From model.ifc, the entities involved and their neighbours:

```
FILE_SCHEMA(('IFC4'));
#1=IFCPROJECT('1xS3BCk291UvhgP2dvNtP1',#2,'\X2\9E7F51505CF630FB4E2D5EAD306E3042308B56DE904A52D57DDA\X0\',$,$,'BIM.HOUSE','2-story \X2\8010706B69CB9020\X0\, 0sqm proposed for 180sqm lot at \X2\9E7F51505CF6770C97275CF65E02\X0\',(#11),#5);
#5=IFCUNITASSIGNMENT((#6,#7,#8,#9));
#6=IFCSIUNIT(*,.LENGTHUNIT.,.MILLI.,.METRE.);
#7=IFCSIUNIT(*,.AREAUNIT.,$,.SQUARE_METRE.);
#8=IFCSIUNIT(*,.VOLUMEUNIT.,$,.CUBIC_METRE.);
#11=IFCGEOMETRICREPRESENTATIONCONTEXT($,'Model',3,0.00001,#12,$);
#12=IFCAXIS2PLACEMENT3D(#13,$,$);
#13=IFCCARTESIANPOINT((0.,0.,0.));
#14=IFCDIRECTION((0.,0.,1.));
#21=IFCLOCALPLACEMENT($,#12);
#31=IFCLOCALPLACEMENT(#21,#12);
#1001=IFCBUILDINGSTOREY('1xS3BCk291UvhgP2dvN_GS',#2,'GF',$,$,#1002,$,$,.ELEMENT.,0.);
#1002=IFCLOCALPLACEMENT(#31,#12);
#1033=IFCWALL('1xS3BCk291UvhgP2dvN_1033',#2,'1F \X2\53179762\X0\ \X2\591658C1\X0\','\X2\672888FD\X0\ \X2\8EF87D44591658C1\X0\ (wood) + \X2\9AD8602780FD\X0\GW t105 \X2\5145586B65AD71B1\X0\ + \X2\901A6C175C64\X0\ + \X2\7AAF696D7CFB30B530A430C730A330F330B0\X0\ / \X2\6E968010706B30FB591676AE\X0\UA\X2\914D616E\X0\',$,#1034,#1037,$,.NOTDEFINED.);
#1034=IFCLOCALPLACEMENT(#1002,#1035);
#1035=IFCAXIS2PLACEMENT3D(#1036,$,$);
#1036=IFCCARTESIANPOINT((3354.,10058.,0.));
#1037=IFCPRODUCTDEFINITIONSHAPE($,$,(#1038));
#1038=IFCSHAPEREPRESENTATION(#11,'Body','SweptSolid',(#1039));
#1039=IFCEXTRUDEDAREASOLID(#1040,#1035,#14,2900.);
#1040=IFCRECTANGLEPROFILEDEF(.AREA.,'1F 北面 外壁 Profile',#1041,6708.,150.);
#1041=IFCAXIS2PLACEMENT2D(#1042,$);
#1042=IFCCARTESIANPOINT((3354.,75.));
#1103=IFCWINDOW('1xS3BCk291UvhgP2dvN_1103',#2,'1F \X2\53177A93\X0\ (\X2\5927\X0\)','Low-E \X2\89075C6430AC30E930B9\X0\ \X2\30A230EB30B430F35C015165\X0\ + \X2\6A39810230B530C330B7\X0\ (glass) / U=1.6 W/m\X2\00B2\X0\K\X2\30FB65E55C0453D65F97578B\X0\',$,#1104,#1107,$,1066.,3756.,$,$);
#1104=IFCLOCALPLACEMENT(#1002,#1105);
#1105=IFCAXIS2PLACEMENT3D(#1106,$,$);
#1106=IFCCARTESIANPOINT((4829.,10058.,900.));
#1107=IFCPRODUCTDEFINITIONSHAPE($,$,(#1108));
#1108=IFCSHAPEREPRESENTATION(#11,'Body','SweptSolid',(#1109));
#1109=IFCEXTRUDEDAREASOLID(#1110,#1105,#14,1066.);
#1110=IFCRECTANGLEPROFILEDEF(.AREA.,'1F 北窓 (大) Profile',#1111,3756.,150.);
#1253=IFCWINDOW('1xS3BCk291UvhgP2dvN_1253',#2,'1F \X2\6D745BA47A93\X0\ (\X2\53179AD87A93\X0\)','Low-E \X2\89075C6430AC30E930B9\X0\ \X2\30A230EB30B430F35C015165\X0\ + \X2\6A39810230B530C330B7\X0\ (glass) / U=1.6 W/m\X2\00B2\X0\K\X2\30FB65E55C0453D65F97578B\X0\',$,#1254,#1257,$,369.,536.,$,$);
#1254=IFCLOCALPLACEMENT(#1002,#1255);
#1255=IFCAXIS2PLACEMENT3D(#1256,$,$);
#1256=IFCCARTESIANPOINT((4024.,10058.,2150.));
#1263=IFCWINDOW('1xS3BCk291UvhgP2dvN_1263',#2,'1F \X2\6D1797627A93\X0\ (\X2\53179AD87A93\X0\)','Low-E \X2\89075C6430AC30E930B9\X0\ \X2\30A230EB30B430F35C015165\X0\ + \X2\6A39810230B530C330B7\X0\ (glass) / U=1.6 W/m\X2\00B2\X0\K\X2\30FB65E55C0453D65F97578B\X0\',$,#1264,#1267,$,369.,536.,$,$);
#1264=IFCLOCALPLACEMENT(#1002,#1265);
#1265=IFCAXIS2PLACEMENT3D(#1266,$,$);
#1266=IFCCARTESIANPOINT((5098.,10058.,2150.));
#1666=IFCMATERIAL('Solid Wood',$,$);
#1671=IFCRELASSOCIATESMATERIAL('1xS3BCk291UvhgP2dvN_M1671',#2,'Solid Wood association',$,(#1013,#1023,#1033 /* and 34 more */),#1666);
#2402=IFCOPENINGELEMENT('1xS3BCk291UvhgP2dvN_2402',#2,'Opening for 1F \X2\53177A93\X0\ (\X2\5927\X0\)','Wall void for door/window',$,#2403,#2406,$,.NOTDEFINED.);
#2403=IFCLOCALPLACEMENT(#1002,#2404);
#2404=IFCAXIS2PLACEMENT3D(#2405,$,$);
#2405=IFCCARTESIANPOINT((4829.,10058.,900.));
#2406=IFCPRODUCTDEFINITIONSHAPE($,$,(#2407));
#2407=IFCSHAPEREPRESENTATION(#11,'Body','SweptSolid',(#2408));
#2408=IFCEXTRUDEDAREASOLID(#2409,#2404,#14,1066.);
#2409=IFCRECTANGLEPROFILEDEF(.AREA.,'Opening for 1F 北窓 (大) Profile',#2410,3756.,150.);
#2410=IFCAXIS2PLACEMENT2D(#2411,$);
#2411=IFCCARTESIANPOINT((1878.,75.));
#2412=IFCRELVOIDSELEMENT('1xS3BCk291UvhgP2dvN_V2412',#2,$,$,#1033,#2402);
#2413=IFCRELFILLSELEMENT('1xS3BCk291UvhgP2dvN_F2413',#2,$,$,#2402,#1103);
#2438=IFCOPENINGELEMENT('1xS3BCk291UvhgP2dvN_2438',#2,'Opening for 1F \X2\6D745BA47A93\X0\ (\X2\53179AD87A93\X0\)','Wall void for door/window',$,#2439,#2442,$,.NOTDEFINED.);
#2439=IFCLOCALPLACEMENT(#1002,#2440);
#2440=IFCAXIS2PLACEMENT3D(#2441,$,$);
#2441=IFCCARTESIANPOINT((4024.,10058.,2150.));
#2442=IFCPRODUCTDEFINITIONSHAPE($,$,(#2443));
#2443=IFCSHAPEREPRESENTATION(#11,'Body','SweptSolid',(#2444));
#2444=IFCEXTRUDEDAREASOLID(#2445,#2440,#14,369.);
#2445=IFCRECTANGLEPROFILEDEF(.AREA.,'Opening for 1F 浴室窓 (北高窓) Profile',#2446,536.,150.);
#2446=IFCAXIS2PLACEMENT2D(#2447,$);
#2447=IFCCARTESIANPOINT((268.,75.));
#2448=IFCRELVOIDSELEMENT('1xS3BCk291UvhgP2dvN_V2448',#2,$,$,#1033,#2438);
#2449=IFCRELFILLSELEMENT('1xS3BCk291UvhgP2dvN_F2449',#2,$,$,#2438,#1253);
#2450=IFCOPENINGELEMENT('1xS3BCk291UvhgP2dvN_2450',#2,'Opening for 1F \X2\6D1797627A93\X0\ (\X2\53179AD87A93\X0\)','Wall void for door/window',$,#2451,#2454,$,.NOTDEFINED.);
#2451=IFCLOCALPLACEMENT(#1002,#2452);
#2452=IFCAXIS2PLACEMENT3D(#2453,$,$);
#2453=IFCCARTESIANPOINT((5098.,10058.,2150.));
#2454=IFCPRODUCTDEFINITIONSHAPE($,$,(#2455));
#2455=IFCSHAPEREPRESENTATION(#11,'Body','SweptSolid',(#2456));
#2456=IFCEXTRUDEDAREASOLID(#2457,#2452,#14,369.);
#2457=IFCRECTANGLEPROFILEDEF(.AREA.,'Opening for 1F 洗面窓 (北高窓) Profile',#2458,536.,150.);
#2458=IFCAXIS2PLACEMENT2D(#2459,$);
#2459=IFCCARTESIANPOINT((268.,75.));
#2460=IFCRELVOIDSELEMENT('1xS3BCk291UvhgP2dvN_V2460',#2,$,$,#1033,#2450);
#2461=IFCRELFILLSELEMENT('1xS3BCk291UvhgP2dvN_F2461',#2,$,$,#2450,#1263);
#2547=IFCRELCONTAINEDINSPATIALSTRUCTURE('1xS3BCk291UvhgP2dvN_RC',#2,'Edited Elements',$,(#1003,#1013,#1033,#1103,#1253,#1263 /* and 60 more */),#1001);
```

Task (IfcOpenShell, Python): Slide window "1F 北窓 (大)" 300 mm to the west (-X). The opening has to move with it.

```python
import ifcopenshell
import ifcopenshell.api.geometry
import ifcopenshell.util.placement

model = ifcopenshell.open("model.ifc")

window = model.by_guid("1xS3BCk291UvhgP2dvN_1103")
opening = window.FillsVoids[0].RelatingOpeningElement
wall = opening.VoidsElements[0].RelatingBuildingElement

wall_matrix = ifcopenshell.util.placement.get_local_placement(wall.ObjectPlacement)
shift = wall_matrix[:3, 0] * -300.0
before = ifcopenshell.util.placement.get_local_placement(window.ObjectPlacement)[:3, 3].copy()

# The window is not placed relative to its opening, so move both.
for product in (opening, window):
    matrix = ifcopenshell.util.placement.get_local_placement(product.ObjectPlacement)
    matrix[:3, 3] += shift
    ifcopenshell.api.geometry.edit_object_placement(model, product=product, matrix=matrix, is_si=False)

after = ifcopenshell.util.placement.get_local_placement(window.ObjectPlacement)[:3, 3]
print("window moved by", (after - before).round(3) + 0.0)

model.write("model_updated.ifc")
```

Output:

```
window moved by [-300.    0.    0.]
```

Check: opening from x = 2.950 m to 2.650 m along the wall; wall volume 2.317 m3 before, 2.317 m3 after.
